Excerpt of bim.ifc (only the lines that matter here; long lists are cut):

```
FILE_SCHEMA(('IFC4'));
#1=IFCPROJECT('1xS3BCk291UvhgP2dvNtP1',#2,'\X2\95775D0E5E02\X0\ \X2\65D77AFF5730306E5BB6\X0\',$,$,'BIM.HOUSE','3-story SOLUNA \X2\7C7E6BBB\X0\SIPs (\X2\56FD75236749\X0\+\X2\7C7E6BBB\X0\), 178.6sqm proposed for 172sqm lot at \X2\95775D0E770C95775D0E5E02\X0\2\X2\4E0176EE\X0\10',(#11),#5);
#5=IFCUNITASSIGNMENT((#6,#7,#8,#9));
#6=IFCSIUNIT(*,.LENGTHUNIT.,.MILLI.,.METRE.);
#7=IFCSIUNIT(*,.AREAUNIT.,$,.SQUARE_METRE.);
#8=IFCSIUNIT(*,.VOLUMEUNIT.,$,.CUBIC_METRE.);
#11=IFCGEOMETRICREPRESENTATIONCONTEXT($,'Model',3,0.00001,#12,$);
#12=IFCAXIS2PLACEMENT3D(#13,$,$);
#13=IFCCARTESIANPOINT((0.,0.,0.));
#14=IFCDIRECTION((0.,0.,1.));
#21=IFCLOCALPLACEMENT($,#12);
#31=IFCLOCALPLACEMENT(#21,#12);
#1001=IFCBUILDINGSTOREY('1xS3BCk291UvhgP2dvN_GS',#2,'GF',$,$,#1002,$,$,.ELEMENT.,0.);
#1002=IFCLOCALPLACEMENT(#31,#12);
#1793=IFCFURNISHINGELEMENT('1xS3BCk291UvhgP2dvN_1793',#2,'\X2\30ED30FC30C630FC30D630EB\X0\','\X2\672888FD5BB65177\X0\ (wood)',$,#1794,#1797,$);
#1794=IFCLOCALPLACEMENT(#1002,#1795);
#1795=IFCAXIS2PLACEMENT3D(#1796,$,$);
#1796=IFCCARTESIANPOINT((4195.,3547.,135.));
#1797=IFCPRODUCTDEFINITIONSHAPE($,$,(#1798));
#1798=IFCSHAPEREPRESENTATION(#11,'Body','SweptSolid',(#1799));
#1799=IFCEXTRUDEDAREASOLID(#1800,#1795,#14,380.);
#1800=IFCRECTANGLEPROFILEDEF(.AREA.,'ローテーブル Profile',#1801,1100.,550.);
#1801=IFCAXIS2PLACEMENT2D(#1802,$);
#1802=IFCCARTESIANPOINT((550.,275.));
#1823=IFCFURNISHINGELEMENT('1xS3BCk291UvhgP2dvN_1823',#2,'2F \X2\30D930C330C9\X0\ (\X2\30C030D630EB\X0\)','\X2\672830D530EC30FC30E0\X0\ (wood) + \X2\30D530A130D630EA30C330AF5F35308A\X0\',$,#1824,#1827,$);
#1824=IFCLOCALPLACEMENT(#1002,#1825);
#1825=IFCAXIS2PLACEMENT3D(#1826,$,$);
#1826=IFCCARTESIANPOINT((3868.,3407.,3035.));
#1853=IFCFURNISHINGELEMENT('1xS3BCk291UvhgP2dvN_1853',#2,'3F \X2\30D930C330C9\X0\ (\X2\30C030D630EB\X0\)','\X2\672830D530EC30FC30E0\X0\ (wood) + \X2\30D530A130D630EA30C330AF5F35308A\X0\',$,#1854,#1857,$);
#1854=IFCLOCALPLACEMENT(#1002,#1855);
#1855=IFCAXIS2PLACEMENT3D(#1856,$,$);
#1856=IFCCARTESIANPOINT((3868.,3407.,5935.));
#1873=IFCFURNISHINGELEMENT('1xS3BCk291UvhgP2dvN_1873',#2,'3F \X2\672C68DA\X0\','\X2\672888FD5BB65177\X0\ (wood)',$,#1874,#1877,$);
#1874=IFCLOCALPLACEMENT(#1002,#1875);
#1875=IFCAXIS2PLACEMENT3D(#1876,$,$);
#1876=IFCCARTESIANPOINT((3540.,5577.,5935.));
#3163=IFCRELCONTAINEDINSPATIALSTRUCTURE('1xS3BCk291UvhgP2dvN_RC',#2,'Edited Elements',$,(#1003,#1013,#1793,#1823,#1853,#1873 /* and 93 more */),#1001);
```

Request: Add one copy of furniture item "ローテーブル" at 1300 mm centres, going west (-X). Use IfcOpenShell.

```python
import numpy as np
import ifcopenshell
import ifcopenshell.api.geometry
import ifcopenshell.api.root
import ifcopenshell.util.element
import ifcopenshell.util.placement

model = ifcopenshell.open("bim.ifc")


def reuse_history(source, copy):
    """copy_class also copies each property set's owner history, people and application; keep the originals."""
    for rel in copy.IsDefinedBy:
        if rel.is_a("IfcRelDefinesByProperties") and (history := rel.RelatingPropertyDefinition.OwnerHistory):
            rel.RelatingPropertyDefinition.OwnerHistory = source.OwnerHistory
            ifcopenshell.util.element.remove_deep2(model, history)


source = model.by_id(1793)
base = ifcopenshell.util.placement.get_local_placement(source.ObjectPlacement)
step = np.array([-1.0, 0.0, 0.0]) * 1300.0

for i in range(1, 2):
    copy = ifcopenshell.api.root.copy_class(model, product=source)
    copy.Representation = ifcopenshell.util.element.copy_deep(
        model, source.Representation, exclude=["IfcGeometricRepresentationContext", "IfcRepresentationMap"]
    )
    reuse_history(source, copy)
    matrix = base.copy()
    matrix[:3, 3] += i * step
    print("added at", matrix[:3, 3].round(3) + 0.0)
    ifcopenshell.api.geometry.edit_object_placement(model, product=copy, matrix=matrix, is_si=False)

model.write("bim_edited.ifc")
```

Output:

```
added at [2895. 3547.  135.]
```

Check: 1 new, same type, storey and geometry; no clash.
